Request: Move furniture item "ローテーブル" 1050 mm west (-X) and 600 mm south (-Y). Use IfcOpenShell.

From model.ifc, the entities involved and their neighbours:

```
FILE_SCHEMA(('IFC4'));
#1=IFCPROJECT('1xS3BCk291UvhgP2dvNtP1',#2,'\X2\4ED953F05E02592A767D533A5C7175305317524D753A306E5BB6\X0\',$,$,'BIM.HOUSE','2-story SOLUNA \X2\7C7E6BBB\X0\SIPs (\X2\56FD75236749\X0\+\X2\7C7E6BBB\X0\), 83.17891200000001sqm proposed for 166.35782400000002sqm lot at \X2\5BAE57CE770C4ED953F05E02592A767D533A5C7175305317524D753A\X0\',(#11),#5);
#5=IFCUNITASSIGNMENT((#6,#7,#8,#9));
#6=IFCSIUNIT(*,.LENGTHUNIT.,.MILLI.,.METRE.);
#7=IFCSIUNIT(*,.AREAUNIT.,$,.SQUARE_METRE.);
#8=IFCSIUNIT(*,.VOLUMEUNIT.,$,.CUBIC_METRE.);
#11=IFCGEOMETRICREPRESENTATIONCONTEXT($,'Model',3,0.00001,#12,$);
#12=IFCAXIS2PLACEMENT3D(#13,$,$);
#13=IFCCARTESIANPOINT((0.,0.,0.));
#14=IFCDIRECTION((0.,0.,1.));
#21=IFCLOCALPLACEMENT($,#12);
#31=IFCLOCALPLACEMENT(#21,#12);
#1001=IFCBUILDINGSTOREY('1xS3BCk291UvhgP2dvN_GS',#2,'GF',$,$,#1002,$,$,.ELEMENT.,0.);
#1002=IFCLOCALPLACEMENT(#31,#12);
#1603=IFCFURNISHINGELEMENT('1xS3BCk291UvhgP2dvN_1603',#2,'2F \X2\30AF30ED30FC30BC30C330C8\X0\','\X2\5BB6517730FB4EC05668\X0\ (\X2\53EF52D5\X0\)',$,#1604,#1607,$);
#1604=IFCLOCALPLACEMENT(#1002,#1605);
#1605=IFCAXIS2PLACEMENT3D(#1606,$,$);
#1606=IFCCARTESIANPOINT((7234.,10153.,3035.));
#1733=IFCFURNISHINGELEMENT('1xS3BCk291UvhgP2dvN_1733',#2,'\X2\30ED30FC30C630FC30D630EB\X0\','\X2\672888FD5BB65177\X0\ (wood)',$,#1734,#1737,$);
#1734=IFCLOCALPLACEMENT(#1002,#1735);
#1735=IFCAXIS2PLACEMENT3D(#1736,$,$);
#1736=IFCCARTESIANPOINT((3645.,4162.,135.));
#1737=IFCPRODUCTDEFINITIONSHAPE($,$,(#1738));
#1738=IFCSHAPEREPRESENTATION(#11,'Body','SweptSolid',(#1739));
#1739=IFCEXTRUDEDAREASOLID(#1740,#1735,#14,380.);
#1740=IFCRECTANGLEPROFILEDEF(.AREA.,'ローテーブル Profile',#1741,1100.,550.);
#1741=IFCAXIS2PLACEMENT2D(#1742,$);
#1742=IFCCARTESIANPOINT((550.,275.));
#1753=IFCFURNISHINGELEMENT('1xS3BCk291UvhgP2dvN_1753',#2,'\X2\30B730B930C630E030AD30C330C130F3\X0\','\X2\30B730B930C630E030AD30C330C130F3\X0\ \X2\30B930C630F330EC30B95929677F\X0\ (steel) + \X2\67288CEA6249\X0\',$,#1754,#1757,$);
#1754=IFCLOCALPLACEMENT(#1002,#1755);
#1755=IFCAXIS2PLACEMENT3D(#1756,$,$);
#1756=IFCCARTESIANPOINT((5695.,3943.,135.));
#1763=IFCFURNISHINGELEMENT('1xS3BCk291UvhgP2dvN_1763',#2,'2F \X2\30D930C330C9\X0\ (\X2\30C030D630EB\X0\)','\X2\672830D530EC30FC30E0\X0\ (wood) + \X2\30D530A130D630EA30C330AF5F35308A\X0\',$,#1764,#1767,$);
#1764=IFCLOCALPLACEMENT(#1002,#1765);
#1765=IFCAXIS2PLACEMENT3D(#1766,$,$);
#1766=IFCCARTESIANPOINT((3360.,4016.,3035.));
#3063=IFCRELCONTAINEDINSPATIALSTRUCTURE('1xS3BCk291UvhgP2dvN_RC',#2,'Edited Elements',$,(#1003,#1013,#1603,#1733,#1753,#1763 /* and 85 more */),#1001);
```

```python
import ifcopenshell
import ifcopenshell.api.geometry
import ifcopenshell.util.placement
import ifcopenshell.util.unit

model = ifcopenshell.open("model.ifc")
unit_scale = ifcopenshell.util.unit.calculate_unit_scale(model)

item = model.by_guid("1xS3BCk291UvhgP2dvN_1733")
matrix = ifcopenshell.util.placement.get_local_placement(item.ObjectPlacement)
matrix[0, 3] -= 1.05 / unit_scale
matrix[1, 3] -= 0.6 / unit_scale
ifcopenshell.api.geometry.edit_object_placement(model, product=item, matrix=matrix, is_si=False)

print(ifcopenshell.util.placement.get_local_placement(item.ObjectPlacement).round(3) + 0.0)

model.write("model_v2.ifc")
```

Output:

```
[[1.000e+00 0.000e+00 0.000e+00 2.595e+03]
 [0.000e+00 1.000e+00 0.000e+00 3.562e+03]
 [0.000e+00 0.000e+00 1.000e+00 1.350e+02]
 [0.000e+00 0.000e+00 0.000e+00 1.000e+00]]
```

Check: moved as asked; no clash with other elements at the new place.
